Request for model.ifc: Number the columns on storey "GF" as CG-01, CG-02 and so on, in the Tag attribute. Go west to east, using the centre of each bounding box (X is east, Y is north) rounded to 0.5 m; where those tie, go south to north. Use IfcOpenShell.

First a look at what the model holds.

```python
import ifcopenshell
import ifcopenshell.util.element
import ifcopenshell.util.placement

model = ifcopenshell.open("model.ifc")
print(model.schema)
storey = next(s for s in model.by_type("IfcBuildingStorey") if s.Name == "GF")
columns = [e for e in ifcopenshell.util.element.get_decomposition(storey) if e.is_a("IfcColumn")]
for e in sorted(columns, key=lambda e: e.id()):
    origin = ifcopenshell.util.placement.get_local_placement(e.ObjectPlacement)[:3, 3]
    print(e.id(), e.Tag, e.Name, origin.round(2) + 0.0, sep=" | ")
```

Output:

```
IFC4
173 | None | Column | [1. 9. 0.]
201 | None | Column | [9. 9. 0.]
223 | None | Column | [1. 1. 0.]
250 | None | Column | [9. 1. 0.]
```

```python
import ifcopenshell
import ifcopenshell.geom
import ifcopenshell.util.element
import ifcopenshell.util.shape

model = ifcopenshell.open("model.ifc")
settings = ifcopenshell.geom.settings()
settings.set("use-world-coords", True)


def centre(element):
    shape = ifcopenshell.geom.create_shape(settings, element)
    return ifcopenshell.util.shape.get_bbox_centroid(shape.geometry)


storey = next(s for s in model.by_type("IfcBuildingStorey") if s.Name == "GF")
columns = [e for e in ifcopenshell.util.element.get_decomposition(storey) if e.is_a("IfcColumn")]

# Insertion points can sit at a corner or the storey origin, so sort by the geometry (in metres).
centres = {e: centre(e) for e in columns}
columns.sort(key=lambda e: (round(centres[e][0] / 0.5), centres[e][1]))

for i, e in enumerate(columns, start=1):
    number = f"CG-{i:02d}"
    e.Tag = number
    print(e.id(), number)

model.write("model_rev.ifc")
```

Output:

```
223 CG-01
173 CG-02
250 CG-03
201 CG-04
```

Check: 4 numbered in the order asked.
